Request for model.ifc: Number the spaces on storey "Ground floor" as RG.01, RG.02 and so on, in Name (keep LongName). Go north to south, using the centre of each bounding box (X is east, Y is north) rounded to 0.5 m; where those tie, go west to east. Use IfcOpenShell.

First a look at what the model holds.

```python
import ifcopenshell
import ifcopenshell.util.element
import ifcopenshell.util.placement

model = ifcopenshell.open("model.ifc")
print(model.schema)
storey = next(s for s in model.by_type("IfcBuildingStorey") if s.Name == "Ground floor")
spaces = [e for e in ifcopenshell.util.element.get_decomposition(storey) if e.is_a("IfcSpace")]
for e in sorted(spaces, key=lambda e: e.id()):
    origin = ifcopenshell.util.placement.get_local_placement(e.ObjectPlacement)[:3, 3]
    print(e.id(), e.Name, e.LongName, origin.round(2) + 0.0, sep=" | ")
```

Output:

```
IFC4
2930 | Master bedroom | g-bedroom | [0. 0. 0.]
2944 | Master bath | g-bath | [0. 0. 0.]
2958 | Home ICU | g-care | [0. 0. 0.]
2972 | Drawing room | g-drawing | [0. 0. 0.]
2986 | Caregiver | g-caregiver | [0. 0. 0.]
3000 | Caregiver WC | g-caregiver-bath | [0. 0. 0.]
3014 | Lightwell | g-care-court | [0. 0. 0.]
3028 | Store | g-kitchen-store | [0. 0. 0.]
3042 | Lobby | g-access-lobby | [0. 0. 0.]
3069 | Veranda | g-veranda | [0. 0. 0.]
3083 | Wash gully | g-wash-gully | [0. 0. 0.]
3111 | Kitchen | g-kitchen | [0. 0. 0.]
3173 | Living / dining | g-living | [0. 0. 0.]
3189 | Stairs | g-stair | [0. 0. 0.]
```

```python
import ifcopenshell
import ifcopenshell.geom
import ifcopenshell.util.element
import ifcopenshell.util.shape

model = ifcopenshell.open("model.ifc")
settings = ifcopenshell.geom.settings()
settings.set("use-world-coords", True)


def centre(element):
    shape = ifcopenshell.geom.create_shape(settings, element)
    return ifcopenshell.util.shape.get_bbox_centroid(shape.geometry)


storey = next(s for s in model.by_type("IfcBuildingStorey") if s.Name == "Ground floor")
spaces = [e for e in ifcopenshell.util.element.get_decomposition(storey) if e.is_a("IfcSpace")]

# Insertion points can sit at a corner or the storey origin, so sort by the geometry (in metres).
centres = {e: centre(e) for e in spaces}
spaces.sort(key=lambda e: (-round(centres[e][1] / 0.5), centres[e][0]))

for i, e in enumerate(spaces, start=1):
    number = f"RG.{i:02d}"
    e.Name = number
    print(e.id(), number)

model.write("model_rev.ifc")
```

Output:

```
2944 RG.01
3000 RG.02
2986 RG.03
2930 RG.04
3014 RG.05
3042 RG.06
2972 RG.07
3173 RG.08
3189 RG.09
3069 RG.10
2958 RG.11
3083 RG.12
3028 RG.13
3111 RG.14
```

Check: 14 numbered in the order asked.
